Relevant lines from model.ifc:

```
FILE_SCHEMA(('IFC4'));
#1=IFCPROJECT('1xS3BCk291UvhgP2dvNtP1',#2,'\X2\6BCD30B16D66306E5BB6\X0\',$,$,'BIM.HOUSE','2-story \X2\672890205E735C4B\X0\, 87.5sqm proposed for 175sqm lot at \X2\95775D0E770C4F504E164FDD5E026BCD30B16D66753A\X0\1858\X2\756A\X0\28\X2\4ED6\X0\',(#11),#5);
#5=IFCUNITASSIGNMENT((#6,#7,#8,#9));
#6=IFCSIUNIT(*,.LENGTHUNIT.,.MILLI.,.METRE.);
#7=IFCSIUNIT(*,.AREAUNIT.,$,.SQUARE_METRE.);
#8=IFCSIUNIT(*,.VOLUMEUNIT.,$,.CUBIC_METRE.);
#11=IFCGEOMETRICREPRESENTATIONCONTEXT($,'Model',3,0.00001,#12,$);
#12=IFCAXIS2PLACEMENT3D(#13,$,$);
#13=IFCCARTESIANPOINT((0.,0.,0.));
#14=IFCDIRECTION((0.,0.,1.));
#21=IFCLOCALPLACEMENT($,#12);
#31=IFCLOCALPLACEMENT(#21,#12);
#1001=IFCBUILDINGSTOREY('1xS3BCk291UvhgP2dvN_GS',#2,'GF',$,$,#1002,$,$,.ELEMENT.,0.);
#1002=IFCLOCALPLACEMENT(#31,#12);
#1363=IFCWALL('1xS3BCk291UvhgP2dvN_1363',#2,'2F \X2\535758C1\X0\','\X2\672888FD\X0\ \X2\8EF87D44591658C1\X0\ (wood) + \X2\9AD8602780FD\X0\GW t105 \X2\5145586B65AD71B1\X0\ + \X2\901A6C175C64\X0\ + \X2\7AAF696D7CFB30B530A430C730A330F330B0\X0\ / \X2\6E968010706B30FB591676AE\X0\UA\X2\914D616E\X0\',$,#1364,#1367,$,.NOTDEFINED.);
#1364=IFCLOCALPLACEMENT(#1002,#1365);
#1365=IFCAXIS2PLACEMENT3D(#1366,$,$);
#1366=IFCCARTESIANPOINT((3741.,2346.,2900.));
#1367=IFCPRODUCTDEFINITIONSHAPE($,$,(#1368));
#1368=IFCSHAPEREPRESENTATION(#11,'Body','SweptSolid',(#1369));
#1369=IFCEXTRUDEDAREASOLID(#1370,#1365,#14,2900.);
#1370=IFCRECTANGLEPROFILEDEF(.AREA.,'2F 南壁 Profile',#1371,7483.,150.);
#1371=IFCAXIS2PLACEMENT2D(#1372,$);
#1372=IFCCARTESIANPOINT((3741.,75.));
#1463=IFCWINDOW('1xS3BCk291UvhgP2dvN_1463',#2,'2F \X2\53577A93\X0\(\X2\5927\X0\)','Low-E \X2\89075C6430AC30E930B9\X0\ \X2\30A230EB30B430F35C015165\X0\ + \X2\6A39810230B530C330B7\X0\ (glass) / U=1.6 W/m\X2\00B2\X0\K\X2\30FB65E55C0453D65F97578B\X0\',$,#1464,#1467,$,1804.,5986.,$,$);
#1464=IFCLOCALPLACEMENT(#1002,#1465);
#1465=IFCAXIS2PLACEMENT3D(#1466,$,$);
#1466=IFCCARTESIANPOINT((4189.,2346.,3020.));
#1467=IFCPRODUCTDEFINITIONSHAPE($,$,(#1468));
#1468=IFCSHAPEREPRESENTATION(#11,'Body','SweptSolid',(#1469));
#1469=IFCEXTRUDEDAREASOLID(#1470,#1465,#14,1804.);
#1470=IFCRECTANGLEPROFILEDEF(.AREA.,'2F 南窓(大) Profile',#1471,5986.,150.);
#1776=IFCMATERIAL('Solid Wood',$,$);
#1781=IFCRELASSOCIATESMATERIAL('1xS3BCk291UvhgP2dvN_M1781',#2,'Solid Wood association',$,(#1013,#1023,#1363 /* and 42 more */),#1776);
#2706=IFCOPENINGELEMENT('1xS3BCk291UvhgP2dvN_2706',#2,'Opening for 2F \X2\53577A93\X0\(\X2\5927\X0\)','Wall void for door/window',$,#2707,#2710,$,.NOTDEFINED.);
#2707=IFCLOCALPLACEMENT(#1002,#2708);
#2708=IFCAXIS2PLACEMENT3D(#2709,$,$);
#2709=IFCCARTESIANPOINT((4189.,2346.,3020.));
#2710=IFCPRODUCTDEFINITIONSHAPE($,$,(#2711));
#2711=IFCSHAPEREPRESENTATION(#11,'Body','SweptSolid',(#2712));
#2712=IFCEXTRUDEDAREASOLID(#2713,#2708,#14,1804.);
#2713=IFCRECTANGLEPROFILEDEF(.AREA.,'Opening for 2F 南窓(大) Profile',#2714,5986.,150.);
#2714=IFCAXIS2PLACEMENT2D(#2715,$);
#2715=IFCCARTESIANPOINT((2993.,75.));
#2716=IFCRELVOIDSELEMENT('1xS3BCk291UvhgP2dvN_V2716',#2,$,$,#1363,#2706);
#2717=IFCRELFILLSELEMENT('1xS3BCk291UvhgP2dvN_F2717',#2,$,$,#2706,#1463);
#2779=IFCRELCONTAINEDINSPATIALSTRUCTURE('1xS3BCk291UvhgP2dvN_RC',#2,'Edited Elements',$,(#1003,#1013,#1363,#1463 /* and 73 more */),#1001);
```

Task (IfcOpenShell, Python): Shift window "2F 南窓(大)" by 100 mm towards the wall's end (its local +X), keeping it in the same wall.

```python
import ifcopenshell
import ifcopenshell.api.geometry
import ifcopenshell.util.placement

model = ifcopenshell.open("model.ifc")

window = model.by_id(1463)
opening = window.FillsVoids[0].RelatingOpeningElement
wall = opening.VoidsElements[0].RelatingBuildingElement

wall_matrix = ifcopenshell.util.placement.get_local_placement(wall.ObjectPlacement)
shift = wall_matrix[:3, 0] * 100.0
before = ifcopenshell.util.placement.get_local_placement(window.ObjectPlacement)[:3, 3].copy()

# The window is not placed relative to its opening, so move both.
for product in (opening, window):
    matrix = ifcopenshell.util.placement.get_local_placement(product.ObjectPlacement)
    matrix[:3, 3] += shift
    ifcopenshell.api.geometry.edit_object_placement(model, product=product, matrix=matrix, is_si=False)

after = ifcopenshell.util.placement.get_local_placement(window.ObjectPlacement)[:3, 3]
print("window moved by", (after - before).round(3) + 0.0)

model.write("model-out.ifc")
```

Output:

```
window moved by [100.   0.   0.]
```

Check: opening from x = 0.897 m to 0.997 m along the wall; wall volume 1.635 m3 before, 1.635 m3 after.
